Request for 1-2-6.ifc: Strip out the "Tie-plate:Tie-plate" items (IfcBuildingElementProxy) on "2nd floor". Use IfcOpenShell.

First a look at what the model holds.

```python
import ifcopenshell
import ifcopenshell.util.element

model = ifcopenshell.open("1-2-6.ifc")
print(model.schema)
storey = next(s for s in model.by_type("IfcBuildingStorey") if s.Name == "2nd floor")
proxies = [e for e in ifcopenshell.util.element.get_decomposition(storey) if e.is_a("IfcBuildingElementProxy")]
seen = {}
for e in proxies:
    element_type = ifcopenshell.util.element.get_type(e)
    name = element_type.Name if element_type not in (None, e) else None
    seen[name] = seen.get(name, 0) + 1
for name, count in sorted(seen.items(), key=str):
    print(count, "x", name)
```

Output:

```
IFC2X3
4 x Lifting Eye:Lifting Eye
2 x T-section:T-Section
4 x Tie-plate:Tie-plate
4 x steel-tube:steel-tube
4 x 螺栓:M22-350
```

```python
import ifcopenshell
import ifcopenshell.api.root
import ifcopenshell.util.element

model = ifcopenshell.open("1-2-6.ifc")

storey = next(s for s in model.by_type("IfcBuildingStorey") if s.Name == "2nd floor")
proxies = [e for e in ifcopenshell.util.element.get_decomposition(storey) if e.is_a("IfcBuildingElementProxy")]
targets = [e for e in proxies if (t := ifcopenshell.util.element.get_type(e)) not in (None, e) and t.Name == "Tie-plate:Tie-plate"]

for e in targets:
    ifcopenshell.api.root.remove_product(model, product=e)
print(len(targets), "removed")

model.write("1-2-6_edited.ifc")
```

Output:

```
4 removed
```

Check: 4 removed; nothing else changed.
